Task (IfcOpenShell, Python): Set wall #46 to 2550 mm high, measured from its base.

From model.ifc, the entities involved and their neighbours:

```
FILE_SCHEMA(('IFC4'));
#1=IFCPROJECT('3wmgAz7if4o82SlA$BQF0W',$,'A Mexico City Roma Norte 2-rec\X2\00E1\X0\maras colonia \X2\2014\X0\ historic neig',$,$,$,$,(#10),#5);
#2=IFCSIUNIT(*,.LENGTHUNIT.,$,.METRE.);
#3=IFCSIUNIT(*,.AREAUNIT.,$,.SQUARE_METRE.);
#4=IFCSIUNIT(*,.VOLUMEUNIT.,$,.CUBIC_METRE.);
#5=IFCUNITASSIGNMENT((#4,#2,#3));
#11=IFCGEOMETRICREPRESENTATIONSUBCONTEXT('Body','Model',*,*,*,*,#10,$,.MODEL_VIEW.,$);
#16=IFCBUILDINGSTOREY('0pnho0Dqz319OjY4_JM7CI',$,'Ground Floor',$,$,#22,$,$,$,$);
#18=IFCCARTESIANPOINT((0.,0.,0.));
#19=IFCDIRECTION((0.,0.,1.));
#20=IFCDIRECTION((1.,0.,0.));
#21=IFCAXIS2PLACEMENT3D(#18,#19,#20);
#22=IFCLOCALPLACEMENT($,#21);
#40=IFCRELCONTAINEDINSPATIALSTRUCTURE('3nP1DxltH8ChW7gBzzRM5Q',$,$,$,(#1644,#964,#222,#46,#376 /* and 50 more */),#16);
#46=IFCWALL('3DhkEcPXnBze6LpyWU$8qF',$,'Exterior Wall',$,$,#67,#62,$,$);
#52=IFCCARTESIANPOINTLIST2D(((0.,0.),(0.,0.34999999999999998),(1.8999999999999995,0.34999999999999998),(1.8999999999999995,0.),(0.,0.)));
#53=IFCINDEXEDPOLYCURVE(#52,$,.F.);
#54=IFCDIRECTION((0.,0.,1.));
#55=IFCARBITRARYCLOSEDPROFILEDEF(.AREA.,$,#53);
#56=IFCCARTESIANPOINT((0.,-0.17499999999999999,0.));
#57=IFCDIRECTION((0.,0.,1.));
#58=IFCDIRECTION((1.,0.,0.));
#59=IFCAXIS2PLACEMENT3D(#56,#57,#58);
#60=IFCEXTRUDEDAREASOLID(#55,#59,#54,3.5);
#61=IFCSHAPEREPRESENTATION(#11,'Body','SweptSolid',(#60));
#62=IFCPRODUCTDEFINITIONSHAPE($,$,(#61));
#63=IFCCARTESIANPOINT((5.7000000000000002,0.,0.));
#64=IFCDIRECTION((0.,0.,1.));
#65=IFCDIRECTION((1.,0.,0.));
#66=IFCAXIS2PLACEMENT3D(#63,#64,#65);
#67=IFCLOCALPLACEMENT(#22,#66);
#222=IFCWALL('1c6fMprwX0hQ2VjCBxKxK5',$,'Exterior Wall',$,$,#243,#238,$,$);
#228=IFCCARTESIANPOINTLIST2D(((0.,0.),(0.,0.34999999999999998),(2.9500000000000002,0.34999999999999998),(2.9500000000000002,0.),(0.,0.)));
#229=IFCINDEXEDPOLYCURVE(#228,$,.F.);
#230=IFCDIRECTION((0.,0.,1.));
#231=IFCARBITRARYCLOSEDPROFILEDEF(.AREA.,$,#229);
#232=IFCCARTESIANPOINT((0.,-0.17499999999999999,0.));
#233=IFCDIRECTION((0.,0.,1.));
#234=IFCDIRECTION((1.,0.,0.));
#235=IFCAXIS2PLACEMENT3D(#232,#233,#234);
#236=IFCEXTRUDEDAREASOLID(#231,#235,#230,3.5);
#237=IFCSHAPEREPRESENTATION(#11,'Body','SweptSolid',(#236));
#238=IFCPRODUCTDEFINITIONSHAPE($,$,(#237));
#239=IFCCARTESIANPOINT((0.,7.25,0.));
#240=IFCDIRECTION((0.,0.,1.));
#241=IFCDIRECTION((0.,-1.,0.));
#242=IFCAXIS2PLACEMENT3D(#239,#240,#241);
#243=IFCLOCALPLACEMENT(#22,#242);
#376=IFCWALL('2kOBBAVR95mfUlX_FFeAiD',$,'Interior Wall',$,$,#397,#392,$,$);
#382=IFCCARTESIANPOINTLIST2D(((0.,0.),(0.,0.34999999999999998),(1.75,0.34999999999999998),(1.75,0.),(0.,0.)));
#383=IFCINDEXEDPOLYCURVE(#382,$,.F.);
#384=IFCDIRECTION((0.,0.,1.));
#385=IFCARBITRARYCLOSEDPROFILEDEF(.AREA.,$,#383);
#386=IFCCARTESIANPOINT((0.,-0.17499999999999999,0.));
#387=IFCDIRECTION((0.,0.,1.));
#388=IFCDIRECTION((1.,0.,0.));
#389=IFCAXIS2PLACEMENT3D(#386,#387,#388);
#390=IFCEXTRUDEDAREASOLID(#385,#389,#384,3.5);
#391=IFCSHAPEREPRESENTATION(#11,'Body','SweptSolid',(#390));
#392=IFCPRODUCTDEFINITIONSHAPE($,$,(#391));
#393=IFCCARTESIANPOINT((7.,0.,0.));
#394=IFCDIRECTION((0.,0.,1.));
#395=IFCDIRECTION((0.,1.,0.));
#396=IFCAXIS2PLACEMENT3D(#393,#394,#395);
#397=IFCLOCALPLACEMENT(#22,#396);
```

```python
import ifcopenshell
import ifcopenshell.geom
import ifcopenshell.util.representation
import ifcopenshell.util.shape

model = ifcopenshell.open("model.ifc")
settings = ifcopenshell.geom.settings()


def volume(element):
    """Net volume in cubic metres, openings subtracted."""
    shape = ifcopenshell.geom.create_shape(settings, element)
    return ifcopenshell.util.shape.get_volume(shape.geometry)


wall = model.by_guid("3DhkEcPXnBze6LpyWU$8qF")
before = volume(wall)

body = ifcopenshell.util.representation.get_representation(wall, "Model", "Body")
solid = body.Items[0]
old_height = solid.Depth
solid.Depth = 2.55
after = volume(wall)

print(f"height {old_height:g} -> {solid.Depth:g}, volume {before:.3f} -> {after:.3f} m3")

model.write("model_updated.ifc")
```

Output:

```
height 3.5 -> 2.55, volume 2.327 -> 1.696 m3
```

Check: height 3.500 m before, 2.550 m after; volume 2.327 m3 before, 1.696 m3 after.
